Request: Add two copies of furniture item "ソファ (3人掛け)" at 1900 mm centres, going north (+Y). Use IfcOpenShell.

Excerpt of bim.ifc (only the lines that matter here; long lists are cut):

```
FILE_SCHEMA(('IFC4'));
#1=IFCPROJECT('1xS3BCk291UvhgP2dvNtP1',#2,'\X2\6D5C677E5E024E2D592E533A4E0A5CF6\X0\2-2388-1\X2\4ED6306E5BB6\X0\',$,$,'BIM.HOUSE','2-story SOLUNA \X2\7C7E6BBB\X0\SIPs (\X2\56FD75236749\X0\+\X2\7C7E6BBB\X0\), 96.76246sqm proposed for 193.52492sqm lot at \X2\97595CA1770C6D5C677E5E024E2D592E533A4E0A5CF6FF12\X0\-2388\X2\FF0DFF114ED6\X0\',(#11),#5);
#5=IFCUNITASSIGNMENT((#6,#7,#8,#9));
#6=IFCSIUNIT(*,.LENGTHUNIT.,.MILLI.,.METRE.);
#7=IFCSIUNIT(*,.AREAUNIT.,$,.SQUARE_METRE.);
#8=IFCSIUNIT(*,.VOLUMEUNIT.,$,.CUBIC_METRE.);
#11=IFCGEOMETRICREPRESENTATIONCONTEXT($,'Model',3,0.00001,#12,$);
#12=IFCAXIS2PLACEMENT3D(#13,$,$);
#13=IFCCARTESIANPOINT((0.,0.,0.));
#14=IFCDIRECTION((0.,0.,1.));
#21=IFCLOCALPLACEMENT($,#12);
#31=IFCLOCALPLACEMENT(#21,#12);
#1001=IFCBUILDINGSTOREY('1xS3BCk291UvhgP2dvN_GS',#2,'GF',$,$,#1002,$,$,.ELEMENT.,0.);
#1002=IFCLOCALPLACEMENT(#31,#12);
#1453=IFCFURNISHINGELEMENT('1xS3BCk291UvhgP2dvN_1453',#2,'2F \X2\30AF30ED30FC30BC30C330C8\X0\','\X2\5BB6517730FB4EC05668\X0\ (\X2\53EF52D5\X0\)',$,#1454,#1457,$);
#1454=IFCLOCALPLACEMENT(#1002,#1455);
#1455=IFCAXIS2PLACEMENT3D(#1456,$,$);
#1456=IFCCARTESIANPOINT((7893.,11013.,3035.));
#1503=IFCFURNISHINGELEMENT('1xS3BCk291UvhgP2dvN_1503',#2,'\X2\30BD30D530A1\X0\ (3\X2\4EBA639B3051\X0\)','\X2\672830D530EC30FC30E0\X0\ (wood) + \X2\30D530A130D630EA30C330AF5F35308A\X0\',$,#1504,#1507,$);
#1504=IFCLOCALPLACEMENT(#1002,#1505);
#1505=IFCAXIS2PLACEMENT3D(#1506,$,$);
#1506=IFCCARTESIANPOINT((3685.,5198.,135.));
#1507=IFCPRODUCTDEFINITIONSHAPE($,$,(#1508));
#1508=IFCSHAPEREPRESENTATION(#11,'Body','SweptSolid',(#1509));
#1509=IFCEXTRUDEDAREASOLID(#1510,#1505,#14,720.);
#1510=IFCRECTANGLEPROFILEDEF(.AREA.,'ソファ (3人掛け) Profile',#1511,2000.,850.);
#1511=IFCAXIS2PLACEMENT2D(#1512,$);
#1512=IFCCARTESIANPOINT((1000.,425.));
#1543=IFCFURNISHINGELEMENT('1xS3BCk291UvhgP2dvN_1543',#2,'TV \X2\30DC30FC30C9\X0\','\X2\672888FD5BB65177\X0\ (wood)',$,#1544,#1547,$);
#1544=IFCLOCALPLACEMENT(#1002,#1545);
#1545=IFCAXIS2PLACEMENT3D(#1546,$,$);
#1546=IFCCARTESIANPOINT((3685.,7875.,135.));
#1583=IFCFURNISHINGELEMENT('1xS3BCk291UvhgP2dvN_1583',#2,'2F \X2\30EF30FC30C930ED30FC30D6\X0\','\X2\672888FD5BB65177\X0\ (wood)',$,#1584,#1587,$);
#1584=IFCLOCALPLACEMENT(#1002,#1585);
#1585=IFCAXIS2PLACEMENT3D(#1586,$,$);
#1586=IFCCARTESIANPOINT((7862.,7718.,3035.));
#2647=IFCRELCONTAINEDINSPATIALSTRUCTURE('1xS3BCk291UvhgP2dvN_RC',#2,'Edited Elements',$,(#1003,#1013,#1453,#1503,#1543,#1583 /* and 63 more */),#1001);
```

```python
import numpy as np
import ifcopenshell
import ifcopenshell.api.geometry
import ifcopenshell.api.root
import ifcopenshell.util.element
import ifcopenshell.util.placement

model = ifcopenshell.open("bim.ifc")


def reuse_history(source, copy):
    """copy_class also copies each property set's owner history, people and application; keep the originals."""
    for rel in copy.IsDefinedBy:
        if rel.is_a("IfcRelDefinesByProperties") and (history := rel.RelatingPropertyDefinition.OwnerHistory):
            rel.RelatingPropertyDefinition.OwnerHistory = source.OwnerHistory
            ifcopenshell.util.element.remove_deep2(model, history)


source = model.by_id(1503)
base = ifcopenshell.util.placement.get_local_placement(source.ObjectPlacement)
step = np.array([0.0, 1.0, 0.0]) * 1900.0

for i in range(1, 3):
    copy = ifcopenshell.api.root.copy_class(model, product=source)
    copy.Representation = ifcopenshell.util.element.copy_deep(
        model, source.Representation, exclude=["IfcGeometricRepresentationContext", "IfcRepresentationMap"]
    )
    reuse_history(source, copy)
    matrix = base.copy()
    matrix[:3, 3] += i * step
    print("added at", matrix[:3, 3].round(3) + 0.0)
    ifcopenshell.api.geometry.edit_object_placement(model, product=copy, matrix=matrix, is_si=False)

model.write("bim_rev.ifc")
```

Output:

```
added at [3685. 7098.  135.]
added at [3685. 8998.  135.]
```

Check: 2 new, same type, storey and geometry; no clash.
